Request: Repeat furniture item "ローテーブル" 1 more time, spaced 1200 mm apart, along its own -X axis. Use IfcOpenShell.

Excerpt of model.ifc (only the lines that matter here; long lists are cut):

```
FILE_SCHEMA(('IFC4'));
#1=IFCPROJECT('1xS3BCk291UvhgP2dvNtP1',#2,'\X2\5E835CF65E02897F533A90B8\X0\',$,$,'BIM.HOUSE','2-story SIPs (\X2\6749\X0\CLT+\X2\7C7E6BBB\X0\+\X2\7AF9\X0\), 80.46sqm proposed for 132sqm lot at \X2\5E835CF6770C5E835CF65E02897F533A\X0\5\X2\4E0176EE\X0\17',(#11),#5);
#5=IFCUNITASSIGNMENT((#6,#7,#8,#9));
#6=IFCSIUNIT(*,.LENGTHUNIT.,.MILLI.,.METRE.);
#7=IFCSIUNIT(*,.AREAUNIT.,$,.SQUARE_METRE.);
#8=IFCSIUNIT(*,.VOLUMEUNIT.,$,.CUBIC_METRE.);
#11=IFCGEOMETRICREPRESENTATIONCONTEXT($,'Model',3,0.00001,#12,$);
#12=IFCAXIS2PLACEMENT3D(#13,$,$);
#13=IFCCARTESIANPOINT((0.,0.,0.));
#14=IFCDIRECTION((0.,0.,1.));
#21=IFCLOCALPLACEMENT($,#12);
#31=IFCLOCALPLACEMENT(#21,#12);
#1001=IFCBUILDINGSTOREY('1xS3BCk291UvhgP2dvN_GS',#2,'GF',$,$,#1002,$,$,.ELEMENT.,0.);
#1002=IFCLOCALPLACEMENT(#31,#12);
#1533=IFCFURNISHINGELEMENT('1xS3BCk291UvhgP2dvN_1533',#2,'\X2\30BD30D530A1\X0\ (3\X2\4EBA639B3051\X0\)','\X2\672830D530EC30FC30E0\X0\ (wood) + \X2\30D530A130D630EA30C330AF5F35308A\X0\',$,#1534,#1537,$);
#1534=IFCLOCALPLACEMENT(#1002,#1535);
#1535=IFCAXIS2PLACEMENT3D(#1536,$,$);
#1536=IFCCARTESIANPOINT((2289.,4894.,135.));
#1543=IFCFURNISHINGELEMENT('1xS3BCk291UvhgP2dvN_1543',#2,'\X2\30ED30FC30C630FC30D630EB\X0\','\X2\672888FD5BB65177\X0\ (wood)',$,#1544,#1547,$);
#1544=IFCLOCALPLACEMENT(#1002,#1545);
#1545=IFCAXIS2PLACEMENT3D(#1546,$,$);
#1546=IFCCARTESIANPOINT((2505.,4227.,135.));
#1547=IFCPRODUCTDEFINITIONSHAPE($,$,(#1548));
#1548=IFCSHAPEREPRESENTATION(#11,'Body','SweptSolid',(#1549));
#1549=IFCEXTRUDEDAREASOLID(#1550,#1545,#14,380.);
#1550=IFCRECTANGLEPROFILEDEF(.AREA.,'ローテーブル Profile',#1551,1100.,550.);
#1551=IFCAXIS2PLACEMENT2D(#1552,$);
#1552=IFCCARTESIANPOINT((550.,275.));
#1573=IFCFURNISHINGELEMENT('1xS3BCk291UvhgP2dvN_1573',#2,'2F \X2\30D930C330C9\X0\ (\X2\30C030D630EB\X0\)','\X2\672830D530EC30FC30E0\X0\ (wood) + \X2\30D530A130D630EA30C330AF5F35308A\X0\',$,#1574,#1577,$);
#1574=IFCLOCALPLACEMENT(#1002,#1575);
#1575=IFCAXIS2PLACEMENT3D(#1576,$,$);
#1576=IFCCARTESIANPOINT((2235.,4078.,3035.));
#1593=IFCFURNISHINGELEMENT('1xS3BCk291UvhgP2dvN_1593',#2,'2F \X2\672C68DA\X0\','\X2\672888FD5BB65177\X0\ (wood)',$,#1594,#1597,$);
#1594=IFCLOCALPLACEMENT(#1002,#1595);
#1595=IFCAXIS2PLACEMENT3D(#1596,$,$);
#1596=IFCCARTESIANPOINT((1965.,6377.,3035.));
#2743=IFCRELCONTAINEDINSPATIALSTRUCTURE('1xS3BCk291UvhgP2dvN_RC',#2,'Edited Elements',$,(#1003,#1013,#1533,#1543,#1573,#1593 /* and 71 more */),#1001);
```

```python
import ifcopenshell
import ifcopenshell.api.geometry
import ifcopenshell.api.root
import ifcopenshell.util.element
import ifcopenshell.util.placement
import ifcopenshell.util.unit

model = ifcopenshell.open("model.ifc")
unit_scale = ifcopenshell.util.unit.calculate_unit_scale(model)


def reuse_history(source, copy):
    """copy_class also copies each property set's owner history, people and application; keep the originals."""
    for rel in copy.IsDefinedBy:
        if rel.is_a("IfcRelDefinesByProperties") and (history := rel.RelatingPropertyDefinition.OwnerHistory):
            rel.RelatingPropertyDefinition.OwnerHistory = source.OwnerHistory
            ifcopenshell.util.element.remove_deep2(model, history)


source = model.by_id(1543)
base = ifcopenshell.util.placement.get_local_placement(source.ObjectPlacement)
step = -base[:3, 0] * 1.2 / unit_scale

for i in range(1, 2):
    copy = ifcopenshell.api.root.copy_class(model, product=source)
    copy.Representation = ifcopenshell.util.element.copy_deep(
        model, source.Representation, exclude=["IfcGeometricRepresentationContext", "IfcRepresentationMap"]
    )
    reuse_history(source, copy)
    matrix = base.copy()
    matrix[:3, 3] += i * step
    print("added at", matrix[:3, 3].round(3) + 0.0)
    ifcopenshell.api.geometry.edit_object_placement(model, product=copy, matrix=matrix, is_si=False)

model.write("model_updated.ifc")
```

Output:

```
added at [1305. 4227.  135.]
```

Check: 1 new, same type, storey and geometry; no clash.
